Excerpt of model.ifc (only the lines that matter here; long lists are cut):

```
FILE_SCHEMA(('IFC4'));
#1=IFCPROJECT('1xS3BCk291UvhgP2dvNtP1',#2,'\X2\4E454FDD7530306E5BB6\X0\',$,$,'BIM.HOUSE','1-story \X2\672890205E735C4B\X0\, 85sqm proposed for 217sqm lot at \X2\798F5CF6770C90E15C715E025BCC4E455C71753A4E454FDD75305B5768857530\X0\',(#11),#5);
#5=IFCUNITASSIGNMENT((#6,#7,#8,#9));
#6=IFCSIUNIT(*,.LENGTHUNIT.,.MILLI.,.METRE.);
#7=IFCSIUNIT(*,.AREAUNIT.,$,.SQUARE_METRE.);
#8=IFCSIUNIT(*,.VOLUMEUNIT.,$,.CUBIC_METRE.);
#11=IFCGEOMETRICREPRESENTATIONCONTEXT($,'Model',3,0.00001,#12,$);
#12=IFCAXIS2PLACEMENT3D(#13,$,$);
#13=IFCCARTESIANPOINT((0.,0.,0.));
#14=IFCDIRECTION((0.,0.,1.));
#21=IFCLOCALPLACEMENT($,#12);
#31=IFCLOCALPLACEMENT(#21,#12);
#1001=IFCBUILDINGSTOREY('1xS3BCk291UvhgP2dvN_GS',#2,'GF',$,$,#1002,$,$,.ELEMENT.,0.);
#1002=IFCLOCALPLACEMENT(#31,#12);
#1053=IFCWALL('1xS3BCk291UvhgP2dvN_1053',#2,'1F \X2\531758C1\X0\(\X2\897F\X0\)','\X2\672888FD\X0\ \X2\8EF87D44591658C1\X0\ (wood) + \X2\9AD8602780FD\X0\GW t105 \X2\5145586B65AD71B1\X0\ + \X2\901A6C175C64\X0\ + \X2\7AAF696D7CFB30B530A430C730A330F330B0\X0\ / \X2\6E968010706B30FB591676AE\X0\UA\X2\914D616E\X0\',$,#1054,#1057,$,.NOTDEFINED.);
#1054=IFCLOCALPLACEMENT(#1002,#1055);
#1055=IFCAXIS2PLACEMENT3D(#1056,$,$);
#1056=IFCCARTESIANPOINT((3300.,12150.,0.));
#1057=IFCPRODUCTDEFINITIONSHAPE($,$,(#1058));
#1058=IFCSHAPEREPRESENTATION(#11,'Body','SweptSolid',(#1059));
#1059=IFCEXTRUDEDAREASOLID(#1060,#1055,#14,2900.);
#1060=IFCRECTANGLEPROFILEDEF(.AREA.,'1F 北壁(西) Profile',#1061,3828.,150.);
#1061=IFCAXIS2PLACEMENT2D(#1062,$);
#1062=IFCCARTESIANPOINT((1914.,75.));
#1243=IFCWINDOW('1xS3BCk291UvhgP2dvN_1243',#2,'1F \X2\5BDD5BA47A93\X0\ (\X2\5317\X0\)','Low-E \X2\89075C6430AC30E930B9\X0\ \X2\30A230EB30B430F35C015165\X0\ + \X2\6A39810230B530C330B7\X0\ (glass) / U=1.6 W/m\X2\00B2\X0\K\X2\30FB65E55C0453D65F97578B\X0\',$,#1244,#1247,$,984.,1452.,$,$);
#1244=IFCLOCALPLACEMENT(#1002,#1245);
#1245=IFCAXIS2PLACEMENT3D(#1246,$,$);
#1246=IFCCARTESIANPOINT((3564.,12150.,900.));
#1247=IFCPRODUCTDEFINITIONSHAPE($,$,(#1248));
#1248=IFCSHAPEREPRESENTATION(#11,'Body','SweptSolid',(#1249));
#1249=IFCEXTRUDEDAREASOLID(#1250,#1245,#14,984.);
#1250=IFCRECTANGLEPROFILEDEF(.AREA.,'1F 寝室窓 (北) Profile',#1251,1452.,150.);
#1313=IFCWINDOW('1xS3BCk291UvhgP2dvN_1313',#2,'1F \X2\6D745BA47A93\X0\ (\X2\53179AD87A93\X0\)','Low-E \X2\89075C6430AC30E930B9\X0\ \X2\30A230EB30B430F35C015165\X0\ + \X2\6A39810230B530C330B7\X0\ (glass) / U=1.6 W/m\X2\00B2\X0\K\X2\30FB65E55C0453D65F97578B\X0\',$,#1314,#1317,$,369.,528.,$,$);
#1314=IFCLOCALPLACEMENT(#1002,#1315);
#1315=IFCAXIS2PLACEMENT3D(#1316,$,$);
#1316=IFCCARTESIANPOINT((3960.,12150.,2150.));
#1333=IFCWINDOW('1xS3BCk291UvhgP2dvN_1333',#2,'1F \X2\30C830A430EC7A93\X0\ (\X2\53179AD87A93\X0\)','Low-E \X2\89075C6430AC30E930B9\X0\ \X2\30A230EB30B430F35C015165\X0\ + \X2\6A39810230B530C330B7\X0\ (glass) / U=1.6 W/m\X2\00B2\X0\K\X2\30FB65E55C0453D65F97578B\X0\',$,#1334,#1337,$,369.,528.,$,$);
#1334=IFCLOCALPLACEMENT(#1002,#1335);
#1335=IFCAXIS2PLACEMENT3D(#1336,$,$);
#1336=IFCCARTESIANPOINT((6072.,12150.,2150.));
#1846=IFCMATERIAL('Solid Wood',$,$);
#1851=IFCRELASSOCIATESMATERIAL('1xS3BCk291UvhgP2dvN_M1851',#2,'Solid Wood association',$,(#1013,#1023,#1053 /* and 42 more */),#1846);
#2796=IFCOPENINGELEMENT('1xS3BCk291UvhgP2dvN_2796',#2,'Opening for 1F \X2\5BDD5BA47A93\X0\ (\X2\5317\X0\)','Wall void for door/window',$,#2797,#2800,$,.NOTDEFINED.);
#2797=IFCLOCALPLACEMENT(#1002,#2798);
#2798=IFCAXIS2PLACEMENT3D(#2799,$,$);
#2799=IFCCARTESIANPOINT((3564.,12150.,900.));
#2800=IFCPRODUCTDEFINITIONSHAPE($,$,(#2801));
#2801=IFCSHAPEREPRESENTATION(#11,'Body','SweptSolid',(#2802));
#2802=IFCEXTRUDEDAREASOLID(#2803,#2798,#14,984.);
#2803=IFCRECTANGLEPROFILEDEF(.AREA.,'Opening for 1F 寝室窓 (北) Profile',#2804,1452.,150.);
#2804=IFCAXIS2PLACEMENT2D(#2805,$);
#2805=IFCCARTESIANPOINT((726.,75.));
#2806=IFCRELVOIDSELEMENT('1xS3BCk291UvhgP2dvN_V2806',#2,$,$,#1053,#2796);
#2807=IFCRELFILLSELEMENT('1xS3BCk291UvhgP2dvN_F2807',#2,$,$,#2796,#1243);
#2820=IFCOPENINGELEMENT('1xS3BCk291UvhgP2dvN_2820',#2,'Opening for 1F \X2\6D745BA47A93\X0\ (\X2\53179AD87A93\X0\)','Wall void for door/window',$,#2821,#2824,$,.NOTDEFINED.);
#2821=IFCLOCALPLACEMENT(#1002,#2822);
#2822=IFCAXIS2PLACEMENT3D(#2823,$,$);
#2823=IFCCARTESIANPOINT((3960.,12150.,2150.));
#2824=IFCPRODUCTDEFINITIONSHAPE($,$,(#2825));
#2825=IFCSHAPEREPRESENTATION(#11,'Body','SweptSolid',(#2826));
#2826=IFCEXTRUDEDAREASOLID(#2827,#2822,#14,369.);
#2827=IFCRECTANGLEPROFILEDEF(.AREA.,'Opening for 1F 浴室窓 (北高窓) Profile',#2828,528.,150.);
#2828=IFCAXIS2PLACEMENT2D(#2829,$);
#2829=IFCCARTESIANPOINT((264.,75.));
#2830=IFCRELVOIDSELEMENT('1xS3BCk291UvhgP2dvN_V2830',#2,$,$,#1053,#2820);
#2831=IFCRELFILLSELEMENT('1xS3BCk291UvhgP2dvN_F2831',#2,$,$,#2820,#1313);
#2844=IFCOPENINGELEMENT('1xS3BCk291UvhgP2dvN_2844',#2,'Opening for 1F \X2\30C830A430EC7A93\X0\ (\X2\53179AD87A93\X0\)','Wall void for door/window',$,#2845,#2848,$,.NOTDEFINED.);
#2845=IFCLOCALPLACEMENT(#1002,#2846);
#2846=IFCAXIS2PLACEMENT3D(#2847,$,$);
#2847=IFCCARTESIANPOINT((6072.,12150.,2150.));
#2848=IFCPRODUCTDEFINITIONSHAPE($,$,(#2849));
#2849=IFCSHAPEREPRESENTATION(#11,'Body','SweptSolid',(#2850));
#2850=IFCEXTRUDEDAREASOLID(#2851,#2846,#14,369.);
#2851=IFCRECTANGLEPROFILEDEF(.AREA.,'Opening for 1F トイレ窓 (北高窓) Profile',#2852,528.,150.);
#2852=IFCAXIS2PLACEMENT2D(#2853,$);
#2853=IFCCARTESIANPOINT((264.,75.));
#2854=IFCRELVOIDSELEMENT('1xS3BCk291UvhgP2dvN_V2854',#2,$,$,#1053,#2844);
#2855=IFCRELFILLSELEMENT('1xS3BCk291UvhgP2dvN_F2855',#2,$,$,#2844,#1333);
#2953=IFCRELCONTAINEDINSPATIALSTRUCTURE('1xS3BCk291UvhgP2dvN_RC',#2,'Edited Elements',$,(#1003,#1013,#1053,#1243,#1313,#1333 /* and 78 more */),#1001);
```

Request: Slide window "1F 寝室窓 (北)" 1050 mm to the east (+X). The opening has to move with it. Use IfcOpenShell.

```python
import ifcopenshell
import ifcopenshell.api.geometry
import ifcopenshell.util.placement

model = ifcopenshell.open("model.ifc")

window = model.by_guid("1xS3BCk291UvhgP2dvN_1243")
opening = window.FillsVoids[0].RelatingOpeningElement
wall = opening.VoidsElements[0].RelatingBuildingElement

wall_matrix = ifcopenshell.util.placement.get_local_placement(wall.ObjectPlacement)
shift = wall_matrix[:3, 0] * 1050.0
before = ifcopenshell.util.placement.get_local_placement(window.ObjectPlacement)[:3, 3].copy()

# The window is not placed relative to its opening, so move both.
for product in (opening, window):
    matrix = ifcopenshell.util.placement.get_local_placement(product.ObjectPlacement)
    matrix[:3, 3] += shift
    ifcopenshell.api.geometry.edit_object_placement(model, product=product, matrix=matrix, is_si=False)

after = ifcopenshell.util.placement.get_local_placement(window.ObjectPlacement)[:3, 3]
print("window moved by", (after - before).round(3) + 0.0)

model.write("model_updated.ifc")
```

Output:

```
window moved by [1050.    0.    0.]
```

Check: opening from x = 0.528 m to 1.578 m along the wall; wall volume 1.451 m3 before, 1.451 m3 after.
